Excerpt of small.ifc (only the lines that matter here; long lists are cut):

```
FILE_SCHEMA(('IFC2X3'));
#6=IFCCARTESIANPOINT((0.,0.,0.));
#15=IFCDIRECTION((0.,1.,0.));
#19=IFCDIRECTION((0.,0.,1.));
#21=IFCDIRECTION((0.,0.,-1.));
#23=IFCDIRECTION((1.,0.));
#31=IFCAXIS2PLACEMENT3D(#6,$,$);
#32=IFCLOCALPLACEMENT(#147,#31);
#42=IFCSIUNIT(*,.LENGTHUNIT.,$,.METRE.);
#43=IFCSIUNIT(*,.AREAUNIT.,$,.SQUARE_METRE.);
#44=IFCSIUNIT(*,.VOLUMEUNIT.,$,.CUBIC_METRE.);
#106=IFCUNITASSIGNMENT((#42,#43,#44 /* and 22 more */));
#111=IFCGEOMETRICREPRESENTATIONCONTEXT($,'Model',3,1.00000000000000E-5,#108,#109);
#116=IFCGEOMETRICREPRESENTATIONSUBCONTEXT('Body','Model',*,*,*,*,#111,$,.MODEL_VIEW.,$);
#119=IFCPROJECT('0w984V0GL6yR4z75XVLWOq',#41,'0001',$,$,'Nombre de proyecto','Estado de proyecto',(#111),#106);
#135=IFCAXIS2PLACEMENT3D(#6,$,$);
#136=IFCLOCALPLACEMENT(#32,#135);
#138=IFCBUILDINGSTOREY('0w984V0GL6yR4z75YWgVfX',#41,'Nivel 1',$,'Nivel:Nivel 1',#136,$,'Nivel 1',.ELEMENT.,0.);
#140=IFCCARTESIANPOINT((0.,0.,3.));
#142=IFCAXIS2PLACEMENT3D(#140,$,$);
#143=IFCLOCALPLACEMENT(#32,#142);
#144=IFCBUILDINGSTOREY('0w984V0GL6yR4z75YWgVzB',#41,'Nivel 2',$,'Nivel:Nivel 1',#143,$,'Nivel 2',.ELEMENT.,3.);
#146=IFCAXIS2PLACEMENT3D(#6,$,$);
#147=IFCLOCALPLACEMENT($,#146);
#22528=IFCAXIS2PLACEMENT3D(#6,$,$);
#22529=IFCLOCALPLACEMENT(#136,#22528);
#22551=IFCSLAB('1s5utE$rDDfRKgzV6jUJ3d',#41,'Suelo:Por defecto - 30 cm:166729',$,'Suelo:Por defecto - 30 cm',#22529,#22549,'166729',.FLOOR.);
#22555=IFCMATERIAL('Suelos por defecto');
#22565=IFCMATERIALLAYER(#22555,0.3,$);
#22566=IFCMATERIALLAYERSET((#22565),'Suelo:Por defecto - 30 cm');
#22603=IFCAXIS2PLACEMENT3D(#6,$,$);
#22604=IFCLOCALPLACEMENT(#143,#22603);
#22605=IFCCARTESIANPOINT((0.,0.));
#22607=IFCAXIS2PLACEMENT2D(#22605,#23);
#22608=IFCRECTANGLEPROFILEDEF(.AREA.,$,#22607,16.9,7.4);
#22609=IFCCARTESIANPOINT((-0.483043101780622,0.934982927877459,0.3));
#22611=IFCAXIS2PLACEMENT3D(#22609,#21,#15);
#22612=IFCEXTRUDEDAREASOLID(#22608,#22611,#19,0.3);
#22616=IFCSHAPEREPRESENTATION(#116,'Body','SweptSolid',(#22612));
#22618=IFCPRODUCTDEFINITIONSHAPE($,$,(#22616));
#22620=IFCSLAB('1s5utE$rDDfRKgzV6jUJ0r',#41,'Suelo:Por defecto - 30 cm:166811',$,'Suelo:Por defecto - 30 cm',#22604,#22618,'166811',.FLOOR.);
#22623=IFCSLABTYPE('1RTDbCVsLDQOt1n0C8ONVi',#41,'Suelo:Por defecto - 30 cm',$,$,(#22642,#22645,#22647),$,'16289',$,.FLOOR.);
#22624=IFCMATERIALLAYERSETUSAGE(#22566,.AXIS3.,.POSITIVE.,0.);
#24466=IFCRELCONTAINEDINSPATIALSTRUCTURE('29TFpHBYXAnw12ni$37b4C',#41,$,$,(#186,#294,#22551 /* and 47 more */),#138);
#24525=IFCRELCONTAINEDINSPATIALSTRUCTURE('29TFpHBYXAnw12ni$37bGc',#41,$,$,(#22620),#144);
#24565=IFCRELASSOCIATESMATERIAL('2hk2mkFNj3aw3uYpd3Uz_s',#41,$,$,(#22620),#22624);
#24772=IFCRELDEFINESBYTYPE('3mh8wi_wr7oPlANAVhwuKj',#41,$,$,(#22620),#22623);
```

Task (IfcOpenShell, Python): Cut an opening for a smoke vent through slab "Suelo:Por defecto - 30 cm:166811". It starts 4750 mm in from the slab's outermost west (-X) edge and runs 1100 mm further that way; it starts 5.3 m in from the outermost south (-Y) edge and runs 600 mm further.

```python
import numpy as np
import ifcopenshell
import ifcopenshell.api.feature
import ifcopenshell.api.geometry
import ifcopenshell.api.root
import ifcopenshell.geom
import ifcopenshell.util.placement
import ifcopenshell.util.representation
import ifcopenshell.util.shape
import ifcopenshell.util.unit

model = ifcopenshell.open("small.ifc")
unit_scale = ifcopenshell.util.unit.calculate_unit_scale(model)
settings = ifcopenshell.geom.settings()


def volume(element):
    """Net volume in cubic metres, openings subtracted."""
    shape = ifcopenshell.geom.create_shape(settings, element)
    return ifcopenshell.util.shape.get_volume(shape.geometry)


slab = model.by_guid("1s5utE$rDDfRKgzV6jUJ0r")
before = volume(slab)

# Extent in the slab's own axes, in metres. The edges named are its -X and -Y sides.
slab_shape = ifcopenshell.geom.create_shape(settings, slab)
vertices = ifcopenshell.util.shape.get_vertices(slab_shape.geometry)
x_min, y_min, bottom = vertices.min(axis=0)
top = vertices[:, 2].max()

opening = ifcopenshell.api.root.create_entity(model, ifc_class="IfcOpeningElement", name="Smoke vent opening")
context = ifcopenshell.util.representation.get_context(model, "Model", "Body", "MODEL_VIEW")
width, depth = 1.1, 0.6
outline = [(0.0, 0.0), (width, 0.0), (width, depth), (0.0, depth), (0.0, 0.0)]
# Overshoot both faces by 50 mm so the cut is clean.
shape = ifcopenshell.api.geometry.add_slab_representation(
    model, context=context, depth=top - bottom + 0.1, polyline=outline
)
ifcopenshell.api.geometry.assign_representation(model, product=opening, representation=shape)

matrix = ifcopenshell.util.placement.get_local_placement(slab.ObjectPlacement)
matrix[:, 3] = matrix @ np.append(np.array([x_min + 4.75, y_min + 5.3, bottom - 0.05]) / unit_scale, 1.0)
ifcopenshell.api.geometry.edit_object_placement(model, product=opening, matrix=matrix, is_si=False)
ifcopenshell.api.feature.add_feature(model, feature=opening, element=slab)

after = volume(slab)

print(f"slab volume {before:.3f} -> {after:.3f} m3")

model.write("small_rev.ifc")
```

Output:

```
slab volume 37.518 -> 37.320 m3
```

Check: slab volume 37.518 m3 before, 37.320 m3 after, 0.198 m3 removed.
